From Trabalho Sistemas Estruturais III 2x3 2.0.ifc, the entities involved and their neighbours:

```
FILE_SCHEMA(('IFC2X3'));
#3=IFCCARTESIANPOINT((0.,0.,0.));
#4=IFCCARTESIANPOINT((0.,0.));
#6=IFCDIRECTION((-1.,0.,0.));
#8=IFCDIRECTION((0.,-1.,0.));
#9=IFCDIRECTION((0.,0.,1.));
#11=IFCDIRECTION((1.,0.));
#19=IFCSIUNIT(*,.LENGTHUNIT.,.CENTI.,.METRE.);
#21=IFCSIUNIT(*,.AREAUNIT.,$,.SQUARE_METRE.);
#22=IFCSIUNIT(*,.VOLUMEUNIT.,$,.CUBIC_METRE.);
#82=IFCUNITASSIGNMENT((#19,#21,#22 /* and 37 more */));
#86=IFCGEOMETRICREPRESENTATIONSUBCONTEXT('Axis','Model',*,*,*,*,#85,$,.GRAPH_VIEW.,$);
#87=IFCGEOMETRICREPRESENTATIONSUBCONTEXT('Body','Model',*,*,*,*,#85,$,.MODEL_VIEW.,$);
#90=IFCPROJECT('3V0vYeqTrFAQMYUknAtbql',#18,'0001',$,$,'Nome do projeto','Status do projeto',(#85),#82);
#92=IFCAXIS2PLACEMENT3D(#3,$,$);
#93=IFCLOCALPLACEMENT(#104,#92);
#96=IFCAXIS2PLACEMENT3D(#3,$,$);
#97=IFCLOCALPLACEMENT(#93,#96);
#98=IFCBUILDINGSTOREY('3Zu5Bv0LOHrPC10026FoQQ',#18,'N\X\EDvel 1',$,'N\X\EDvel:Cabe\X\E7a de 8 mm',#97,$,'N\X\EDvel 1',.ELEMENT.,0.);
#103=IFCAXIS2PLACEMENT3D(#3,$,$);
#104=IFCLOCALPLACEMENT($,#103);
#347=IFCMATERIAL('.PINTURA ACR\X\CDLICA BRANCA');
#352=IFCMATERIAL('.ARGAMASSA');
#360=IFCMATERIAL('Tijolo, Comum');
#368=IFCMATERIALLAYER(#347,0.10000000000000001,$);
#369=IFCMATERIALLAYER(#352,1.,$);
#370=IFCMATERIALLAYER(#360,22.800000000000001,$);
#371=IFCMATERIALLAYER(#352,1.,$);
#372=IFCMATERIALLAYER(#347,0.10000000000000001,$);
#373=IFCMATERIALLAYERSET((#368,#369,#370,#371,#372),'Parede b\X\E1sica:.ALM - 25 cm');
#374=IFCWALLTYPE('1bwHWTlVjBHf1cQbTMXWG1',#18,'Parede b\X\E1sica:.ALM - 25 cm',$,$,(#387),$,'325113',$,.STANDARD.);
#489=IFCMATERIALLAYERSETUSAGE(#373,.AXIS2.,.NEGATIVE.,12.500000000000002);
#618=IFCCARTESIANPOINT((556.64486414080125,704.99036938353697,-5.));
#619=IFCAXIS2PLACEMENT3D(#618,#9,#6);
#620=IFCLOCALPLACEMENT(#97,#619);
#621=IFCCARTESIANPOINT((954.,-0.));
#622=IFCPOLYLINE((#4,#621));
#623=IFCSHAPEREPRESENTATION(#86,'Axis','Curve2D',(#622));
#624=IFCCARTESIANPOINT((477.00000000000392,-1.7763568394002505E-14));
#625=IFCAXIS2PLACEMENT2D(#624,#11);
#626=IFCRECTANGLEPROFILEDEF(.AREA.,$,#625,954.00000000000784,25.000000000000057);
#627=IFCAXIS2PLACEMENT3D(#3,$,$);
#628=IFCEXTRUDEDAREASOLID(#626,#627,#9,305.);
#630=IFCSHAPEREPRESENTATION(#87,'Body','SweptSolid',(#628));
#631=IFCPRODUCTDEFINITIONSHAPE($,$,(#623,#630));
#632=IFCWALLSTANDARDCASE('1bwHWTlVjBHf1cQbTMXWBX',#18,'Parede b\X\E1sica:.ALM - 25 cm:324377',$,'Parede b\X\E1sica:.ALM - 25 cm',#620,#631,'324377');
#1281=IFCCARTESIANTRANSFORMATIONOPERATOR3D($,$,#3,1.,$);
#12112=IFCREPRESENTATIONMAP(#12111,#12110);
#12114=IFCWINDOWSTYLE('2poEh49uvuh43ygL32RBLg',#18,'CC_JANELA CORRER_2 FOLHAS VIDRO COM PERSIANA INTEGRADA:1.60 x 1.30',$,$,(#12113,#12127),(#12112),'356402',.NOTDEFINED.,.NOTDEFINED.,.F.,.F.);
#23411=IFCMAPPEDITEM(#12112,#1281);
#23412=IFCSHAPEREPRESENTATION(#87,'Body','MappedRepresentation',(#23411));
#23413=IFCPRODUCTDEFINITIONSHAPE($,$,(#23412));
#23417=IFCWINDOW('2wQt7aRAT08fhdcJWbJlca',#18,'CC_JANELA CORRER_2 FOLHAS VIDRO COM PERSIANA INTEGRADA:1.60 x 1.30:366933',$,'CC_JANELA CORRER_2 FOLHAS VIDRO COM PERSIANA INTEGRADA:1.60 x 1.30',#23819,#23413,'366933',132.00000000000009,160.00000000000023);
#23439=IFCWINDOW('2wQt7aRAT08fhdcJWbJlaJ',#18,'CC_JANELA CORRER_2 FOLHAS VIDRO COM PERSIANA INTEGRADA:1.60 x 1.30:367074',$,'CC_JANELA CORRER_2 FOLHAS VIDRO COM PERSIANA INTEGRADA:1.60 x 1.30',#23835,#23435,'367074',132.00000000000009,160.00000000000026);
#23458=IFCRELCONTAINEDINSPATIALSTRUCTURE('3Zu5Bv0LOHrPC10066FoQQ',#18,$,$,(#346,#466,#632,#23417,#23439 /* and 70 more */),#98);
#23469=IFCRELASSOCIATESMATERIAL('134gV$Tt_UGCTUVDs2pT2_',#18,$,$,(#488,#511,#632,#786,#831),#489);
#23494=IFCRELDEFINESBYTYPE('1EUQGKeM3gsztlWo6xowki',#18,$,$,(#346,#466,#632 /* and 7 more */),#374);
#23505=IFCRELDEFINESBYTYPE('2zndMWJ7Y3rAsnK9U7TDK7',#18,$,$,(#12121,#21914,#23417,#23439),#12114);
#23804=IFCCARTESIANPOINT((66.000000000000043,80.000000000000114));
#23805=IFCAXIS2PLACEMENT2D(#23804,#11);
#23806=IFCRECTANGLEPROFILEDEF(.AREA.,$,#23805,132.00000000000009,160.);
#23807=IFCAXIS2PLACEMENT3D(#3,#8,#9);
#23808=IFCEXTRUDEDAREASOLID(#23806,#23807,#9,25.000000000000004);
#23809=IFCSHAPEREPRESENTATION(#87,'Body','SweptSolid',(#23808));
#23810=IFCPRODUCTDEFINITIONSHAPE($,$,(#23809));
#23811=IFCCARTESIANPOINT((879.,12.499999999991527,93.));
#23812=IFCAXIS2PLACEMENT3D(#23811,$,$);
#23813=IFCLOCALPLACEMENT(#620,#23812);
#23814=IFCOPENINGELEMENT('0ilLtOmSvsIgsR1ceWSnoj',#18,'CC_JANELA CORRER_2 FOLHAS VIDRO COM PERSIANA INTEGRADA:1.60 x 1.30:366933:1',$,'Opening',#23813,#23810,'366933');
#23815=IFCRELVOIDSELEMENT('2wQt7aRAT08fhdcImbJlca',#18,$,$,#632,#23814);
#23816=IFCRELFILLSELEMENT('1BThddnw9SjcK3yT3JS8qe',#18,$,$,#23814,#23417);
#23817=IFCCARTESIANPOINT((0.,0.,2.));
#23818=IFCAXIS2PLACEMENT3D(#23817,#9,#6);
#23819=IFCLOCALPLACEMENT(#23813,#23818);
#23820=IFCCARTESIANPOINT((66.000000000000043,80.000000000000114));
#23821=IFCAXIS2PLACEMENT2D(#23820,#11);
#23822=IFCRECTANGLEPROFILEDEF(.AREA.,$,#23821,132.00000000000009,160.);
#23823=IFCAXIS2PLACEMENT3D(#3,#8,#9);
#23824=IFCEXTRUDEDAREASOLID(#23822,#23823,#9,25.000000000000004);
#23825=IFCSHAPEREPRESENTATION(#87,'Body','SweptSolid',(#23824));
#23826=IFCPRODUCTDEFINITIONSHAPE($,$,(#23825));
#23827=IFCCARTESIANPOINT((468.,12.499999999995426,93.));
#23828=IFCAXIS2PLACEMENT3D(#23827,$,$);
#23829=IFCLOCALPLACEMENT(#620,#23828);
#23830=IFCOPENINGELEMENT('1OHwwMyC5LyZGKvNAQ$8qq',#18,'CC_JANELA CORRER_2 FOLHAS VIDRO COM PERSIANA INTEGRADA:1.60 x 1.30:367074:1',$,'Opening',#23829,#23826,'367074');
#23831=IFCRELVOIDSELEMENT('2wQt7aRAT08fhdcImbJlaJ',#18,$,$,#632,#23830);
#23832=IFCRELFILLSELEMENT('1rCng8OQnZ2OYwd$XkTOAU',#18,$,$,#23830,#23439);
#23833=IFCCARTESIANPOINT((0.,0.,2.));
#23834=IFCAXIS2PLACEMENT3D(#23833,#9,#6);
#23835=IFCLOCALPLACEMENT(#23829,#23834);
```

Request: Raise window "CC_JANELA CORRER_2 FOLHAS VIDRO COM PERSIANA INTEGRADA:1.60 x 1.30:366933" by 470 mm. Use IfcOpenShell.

```python
import numpy as np
import ifcopenshell
import ifcopenshell.api.geometry
import ifcopenshell.util.placement
import ifcopenshell.util.unit

model = ifcopenshell.open("Trabalho Sistemas Estruturais III 2x3 2.0.ifc")
unit_scale = ifcopenshell.util.unit.calculate_unit_scale(model)

window = model.by_guid("2wQt7aRAT08fhdcJWbJlca")
opening = window.FillsVoids[0].RelatingOpeningElement
dz = 0.47 / unit_scale

shift = np.array([0.0, 0.0, dz])
# The window is placed relative to its opening, so it follows when the opening moves.
matrix = ifcopenshell.util.placement.get_local_placement(opening.ObjectPlacement)
matrix[:3, 3] += shift
ifcopenshell.api.geometry.edit_object_placement(
    model, product=opening, matrix=matrix, is_si=False, should_transform_children=True
)

print(f"moved by {dz * unit_scale:+.3f} m")

model.write("Trabalho Sistemas Estruturais III 2x3 2.0_updated.ifc")
```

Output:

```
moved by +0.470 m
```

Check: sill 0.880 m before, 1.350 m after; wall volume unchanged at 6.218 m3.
